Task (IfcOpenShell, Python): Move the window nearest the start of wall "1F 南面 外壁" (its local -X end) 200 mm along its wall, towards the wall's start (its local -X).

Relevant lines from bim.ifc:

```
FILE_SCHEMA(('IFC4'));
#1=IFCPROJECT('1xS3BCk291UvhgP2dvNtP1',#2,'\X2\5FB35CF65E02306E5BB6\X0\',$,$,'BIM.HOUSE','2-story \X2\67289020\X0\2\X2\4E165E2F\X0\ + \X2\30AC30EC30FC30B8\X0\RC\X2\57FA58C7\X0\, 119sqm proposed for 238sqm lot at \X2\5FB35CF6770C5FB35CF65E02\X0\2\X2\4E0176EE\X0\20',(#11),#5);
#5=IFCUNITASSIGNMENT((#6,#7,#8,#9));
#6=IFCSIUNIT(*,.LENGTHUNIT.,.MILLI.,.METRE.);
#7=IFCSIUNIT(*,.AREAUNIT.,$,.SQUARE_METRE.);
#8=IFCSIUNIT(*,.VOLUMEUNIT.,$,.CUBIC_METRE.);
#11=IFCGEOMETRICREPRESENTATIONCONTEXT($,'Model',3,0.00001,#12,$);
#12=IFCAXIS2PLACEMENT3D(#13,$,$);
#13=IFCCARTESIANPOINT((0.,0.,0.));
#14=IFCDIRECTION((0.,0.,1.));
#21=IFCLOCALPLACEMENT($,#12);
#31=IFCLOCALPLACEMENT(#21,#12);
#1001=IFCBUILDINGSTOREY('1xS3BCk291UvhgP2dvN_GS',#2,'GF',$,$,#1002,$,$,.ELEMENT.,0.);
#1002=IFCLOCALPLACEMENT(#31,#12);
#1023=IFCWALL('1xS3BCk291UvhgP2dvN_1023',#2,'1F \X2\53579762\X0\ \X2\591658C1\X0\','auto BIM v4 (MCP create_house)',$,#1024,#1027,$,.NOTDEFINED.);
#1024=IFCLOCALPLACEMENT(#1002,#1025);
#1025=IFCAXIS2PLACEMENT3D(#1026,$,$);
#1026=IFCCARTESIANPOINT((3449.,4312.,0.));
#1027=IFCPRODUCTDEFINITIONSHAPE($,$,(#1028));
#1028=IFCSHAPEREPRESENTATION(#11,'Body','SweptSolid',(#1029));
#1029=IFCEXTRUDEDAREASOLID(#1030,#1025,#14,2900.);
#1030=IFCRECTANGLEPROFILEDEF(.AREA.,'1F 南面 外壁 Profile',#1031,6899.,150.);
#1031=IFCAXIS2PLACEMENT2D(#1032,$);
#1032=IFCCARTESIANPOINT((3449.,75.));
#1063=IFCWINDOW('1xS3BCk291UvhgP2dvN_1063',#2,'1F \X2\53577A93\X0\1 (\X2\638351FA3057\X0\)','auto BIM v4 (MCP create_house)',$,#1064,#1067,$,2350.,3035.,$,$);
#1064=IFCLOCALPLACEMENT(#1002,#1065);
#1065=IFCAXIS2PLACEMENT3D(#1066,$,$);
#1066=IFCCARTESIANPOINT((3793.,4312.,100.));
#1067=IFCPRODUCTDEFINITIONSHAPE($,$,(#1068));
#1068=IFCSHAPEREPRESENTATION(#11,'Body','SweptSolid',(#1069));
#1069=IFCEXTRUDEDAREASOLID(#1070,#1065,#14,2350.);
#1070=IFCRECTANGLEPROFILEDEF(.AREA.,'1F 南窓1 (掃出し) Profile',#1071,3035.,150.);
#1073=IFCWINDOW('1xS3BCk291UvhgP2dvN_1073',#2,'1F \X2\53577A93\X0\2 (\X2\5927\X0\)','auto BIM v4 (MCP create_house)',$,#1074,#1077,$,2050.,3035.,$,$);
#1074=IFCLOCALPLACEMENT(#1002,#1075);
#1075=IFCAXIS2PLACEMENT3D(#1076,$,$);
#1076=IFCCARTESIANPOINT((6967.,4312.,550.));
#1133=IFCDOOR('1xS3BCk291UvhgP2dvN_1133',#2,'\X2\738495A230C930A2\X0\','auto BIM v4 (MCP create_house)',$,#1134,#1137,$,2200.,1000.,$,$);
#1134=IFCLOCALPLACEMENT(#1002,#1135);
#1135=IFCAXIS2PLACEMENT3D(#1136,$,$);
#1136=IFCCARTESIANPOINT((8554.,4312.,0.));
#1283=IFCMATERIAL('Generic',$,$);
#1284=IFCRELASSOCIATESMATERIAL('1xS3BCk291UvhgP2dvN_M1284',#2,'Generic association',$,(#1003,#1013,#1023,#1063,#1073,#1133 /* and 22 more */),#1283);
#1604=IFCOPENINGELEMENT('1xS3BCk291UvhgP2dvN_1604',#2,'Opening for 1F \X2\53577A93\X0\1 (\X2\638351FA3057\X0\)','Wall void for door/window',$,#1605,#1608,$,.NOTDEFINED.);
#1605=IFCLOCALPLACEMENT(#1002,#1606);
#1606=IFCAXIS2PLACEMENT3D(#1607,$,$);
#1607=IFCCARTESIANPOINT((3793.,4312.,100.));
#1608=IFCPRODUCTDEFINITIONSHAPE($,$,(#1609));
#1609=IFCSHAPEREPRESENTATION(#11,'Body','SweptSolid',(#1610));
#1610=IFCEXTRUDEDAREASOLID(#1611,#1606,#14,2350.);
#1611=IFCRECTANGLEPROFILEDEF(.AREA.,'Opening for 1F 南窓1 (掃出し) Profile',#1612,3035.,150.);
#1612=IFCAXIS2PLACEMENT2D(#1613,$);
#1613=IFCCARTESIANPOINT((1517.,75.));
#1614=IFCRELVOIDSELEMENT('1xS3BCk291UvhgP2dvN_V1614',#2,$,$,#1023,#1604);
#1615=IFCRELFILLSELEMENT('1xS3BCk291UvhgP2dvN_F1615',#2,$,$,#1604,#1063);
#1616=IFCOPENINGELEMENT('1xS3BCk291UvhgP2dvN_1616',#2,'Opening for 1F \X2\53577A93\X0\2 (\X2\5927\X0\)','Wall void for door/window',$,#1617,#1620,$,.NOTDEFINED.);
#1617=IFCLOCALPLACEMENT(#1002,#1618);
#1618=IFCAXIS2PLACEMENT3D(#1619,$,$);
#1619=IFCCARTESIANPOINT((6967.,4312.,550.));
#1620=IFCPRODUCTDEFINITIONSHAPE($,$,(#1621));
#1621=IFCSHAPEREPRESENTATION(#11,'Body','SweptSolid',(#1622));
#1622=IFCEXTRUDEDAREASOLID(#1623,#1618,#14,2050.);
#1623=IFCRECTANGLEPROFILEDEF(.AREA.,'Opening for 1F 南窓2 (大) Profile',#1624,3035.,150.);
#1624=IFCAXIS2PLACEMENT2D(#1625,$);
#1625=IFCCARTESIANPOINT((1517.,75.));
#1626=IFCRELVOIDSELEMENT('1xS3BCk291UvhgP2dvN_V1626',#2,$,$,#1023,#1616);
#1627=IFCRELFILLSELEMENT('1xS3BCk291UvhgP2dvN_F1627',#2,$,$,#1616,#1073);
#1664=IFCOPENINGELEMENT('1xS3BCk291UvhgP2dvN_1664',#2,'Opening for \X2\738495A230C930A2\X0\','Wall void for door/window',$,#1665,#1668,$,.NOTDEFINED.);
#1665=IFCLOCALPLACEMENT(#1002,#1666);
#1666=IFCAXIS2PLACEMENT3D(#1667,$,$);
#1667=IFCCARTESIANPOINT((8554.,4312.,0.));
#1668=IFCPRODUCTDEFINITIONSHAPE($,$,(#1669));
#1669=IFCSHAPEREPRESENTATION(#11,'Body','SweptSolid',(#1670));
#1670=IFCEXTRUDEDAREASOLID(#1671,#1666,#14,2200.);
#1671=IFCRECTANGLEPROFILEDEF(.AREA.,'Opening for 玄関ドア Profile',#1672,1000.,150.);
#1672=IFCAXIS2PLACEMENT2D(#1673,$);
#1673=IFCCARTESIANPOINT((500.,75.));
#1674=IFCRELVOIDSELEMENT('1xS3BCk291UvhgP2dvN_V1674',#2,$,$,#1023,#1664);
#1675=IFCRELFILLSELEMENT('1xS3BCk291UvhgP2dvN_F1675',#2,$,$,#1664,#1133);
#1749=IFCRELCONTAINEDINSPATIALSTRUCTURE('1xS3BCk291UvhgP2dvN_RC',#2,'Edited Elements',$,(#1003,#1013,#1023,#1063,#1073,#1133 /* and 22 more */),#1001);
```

```python
import ifcopenshell
import ifcopenshell.api.geometry
import ifcopenshell.util.placement

model = ifcopenshell.open("bim.ifc")

window = model.by_guid("1xS3BCk291UvhgP2dvN_1063")
opening = window.FillsVoids[0].RelatingOpeningElement
wall = opening.VoidsElements[0].RelatingBuildingElement

wall_matrix = ifcopenshell.util.placement.get_local_placement(wall.ObjectPlacement)
shift = wall_matrix[:3, 0] * -200.0
before = ifcopenshell.util.placement.get_local_placement(window.ObjectPlacement)[:3, 3].copy()

# The window is not placed relative to its opening, so move both.
for product in (opening, window):
    matrix = ifcopenshell.util.placement.get_local_placement(product.ObjectPlacement)
    matrix[:3, 3] += shift
    ifcopenshell.api.geometry.edit_object_placement(model, product=product, matrix=matrix, is_si=False)

after = ifcopenshell.util.placement.get_local_placement(window.ObjectPlacement)[:3, 3]
print("window moved by", (after - before).round(3) + 0.0)

model.write("bim_v2.ifc")
```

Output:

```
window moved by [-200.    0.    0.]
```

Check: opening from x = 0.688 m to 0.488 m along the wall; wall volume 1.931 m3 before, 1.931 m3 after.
